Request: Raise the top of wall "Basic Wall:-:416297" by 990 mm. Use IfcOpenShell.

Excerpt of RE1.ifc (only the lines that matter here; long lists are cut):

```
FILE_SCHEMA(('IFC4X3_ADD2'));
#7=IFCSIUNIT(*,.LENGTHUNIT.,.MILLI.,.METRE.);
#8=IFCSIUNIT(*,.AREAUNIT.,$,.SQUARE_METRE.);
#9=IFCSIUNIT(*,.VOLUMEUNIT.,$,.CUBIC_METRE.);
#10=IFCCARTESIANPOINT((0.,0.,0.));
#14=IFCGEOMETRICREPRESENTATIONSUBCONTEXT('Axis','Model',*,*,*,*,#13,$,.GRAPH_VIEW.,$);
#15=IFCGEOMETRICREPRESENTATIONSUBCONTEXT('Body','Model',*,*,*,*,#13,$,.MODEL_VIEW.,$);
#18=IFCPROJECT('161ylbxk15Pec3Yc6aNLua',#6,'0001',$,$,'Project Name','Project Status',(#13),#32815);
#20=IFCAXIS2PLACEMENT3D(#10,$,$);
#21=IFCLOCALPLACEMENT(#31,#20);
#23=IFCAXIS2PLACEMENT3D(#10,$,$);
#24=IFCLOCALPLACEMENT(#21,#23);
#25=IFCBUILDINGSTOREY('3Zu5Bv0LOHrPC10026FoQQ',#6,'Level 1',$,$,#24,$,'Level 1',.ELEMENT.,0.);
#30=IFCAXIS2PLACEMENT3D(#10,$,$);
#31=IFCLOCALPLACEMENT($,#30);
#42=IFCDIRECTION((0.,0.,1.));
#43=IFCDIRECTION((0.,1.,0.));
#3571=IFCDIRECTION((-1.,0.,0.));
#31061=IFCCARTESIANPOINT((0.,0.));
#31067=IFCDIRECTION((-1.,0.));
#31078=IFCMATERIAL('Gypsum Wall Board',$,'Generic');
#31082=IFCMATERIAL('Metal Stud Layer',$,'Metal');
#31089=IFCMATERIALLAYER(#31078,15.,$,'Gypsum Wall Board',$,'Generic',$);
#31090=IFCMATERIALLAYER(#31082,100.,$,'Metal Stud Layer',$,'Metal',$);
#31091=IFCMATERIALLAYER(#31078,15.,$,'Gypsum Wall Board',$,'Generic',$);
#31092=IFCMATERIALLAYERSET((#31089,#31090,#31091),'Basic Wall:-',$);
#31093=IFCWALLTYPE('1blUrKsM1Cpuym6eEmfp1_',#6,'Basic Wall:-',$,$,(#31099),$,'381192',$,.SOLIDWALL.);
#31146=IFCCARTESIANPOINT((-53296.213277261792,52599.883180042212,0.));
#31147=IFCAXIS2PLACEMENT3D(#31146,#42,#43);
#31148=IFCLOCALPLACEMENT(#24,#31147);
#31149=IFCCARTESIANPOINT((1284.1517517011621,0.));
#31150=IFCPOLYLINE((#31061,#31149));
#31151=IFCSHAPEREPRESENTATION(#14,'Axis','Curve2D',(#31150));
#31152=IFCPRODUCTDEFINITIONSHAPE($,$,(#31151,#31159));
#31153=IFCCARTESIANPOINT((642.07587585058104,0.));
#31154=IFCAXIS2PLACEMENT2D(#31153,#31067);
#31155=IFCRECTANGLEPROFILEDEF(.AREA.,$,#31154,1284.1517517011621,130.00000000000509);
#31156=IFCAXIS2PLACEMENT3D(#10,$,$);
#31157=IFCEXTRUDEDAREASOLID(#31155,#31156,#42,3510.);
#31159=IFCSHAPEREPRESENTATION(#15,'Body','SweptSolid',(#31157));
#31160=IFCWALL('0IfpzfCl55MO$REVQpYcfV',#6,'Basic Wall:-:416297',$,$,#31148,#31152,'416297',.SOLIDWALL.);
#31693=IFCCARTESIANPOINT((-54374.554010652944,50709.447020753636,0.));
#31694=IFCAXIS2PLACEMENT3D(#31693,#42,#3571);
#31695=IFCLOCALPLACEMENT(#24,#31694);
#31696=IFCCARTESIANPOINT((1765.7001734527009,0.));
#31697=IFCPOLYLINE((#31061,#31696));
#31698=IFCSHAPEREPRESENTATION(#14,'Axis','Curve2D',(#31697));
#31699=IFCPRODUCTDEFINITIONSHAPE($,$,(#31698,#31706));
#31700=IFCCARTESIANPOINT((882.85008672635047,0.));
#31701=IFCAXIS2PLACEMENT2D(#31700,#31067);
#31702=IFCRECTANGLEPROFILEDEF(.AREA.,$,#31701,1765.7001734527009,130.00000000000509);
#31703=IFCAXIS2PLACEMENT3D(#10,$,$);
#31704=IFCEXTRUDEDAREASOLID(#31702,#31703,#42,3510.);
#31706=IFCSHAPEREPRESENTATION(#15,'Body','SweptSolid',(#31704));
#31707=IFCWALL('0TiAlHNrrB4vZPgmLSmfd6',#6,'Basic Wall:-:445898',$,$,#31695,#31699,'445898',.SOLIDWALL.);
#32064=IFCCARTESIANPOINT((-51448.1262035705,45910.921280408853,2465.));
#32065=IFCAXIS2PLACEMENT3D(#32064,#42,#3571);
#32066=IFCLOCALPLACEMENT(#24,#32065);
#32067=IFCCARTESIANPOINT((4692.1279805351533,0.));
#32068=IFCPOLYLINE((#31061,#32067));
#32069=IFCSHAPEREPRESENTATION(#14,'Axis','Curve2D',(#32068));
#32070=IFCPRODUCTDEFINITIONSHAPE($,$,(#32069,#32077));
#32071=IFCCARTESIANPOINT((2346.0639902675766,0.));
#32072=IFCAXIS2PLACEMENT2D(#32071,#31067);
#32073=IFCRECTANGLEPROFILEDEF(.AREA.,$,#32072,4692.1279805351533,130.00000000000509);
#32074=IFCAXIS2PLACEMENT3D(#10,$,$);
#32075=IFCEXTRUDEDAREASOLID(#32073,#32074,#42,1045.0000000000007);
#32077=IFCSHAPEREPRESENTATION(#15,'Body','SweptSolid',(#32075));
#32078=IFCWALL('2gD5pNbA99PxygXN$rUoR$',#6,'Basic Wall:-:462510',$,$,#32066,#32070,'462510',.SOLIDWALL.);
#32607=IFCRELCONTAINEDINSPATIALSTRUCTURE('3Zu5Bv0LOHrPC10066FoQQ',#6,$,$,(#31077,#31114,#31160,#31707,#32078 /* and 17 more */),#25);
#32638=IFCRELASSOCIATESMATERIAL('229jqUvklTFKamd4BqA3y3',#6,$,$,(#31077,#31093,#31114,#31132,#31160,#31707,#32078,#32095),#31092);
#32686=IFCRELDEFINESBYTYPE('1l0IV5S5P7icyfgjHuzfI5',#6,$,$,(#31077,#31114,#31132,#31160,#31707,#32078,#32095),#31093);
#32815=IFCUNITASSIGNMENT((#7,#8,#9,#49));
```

```python
import ifcopenshell
import ifcopenshell.geom
import ifcopenshell.util.representation
import ifcopenshell.util.shape
import ifcopenshell.util.unit

model = ifcopenshell.open("RE1.ifc")
unit_scale = ifcopenshell.util.unit.calculate_unit_scale(model)
settings = ifcopenshell.geom.settings()


def volume(element):
    """Net volume in cubic metres, openings subtracted."""
    shape = ifcopenshell.geom.create_shape(settings, element)
    return ifcopenshell.util.shape.get_volume(shape.geometry)


wall = model.by_guid("0IfpzfCl55MO$REVQpYcfV")
before = volume(wall)

body = ifcopenshell.util.representation.get_representation(wall, "Model", "Body")
solid = body.Items[0]
old_height = solid.Depth
solid.Depth += 0.99 / unit_scale
after = volume(wall)

print(f"height {old_height:g} -> {solid.Depth:g}, volume {before:.3f} -> {after:.3f} m3")

model.write("RE1_rev.ifc")
```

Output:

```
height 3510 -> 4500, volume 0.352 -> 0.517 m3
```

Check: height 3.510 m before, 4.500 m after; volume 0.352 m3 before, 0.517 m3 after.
